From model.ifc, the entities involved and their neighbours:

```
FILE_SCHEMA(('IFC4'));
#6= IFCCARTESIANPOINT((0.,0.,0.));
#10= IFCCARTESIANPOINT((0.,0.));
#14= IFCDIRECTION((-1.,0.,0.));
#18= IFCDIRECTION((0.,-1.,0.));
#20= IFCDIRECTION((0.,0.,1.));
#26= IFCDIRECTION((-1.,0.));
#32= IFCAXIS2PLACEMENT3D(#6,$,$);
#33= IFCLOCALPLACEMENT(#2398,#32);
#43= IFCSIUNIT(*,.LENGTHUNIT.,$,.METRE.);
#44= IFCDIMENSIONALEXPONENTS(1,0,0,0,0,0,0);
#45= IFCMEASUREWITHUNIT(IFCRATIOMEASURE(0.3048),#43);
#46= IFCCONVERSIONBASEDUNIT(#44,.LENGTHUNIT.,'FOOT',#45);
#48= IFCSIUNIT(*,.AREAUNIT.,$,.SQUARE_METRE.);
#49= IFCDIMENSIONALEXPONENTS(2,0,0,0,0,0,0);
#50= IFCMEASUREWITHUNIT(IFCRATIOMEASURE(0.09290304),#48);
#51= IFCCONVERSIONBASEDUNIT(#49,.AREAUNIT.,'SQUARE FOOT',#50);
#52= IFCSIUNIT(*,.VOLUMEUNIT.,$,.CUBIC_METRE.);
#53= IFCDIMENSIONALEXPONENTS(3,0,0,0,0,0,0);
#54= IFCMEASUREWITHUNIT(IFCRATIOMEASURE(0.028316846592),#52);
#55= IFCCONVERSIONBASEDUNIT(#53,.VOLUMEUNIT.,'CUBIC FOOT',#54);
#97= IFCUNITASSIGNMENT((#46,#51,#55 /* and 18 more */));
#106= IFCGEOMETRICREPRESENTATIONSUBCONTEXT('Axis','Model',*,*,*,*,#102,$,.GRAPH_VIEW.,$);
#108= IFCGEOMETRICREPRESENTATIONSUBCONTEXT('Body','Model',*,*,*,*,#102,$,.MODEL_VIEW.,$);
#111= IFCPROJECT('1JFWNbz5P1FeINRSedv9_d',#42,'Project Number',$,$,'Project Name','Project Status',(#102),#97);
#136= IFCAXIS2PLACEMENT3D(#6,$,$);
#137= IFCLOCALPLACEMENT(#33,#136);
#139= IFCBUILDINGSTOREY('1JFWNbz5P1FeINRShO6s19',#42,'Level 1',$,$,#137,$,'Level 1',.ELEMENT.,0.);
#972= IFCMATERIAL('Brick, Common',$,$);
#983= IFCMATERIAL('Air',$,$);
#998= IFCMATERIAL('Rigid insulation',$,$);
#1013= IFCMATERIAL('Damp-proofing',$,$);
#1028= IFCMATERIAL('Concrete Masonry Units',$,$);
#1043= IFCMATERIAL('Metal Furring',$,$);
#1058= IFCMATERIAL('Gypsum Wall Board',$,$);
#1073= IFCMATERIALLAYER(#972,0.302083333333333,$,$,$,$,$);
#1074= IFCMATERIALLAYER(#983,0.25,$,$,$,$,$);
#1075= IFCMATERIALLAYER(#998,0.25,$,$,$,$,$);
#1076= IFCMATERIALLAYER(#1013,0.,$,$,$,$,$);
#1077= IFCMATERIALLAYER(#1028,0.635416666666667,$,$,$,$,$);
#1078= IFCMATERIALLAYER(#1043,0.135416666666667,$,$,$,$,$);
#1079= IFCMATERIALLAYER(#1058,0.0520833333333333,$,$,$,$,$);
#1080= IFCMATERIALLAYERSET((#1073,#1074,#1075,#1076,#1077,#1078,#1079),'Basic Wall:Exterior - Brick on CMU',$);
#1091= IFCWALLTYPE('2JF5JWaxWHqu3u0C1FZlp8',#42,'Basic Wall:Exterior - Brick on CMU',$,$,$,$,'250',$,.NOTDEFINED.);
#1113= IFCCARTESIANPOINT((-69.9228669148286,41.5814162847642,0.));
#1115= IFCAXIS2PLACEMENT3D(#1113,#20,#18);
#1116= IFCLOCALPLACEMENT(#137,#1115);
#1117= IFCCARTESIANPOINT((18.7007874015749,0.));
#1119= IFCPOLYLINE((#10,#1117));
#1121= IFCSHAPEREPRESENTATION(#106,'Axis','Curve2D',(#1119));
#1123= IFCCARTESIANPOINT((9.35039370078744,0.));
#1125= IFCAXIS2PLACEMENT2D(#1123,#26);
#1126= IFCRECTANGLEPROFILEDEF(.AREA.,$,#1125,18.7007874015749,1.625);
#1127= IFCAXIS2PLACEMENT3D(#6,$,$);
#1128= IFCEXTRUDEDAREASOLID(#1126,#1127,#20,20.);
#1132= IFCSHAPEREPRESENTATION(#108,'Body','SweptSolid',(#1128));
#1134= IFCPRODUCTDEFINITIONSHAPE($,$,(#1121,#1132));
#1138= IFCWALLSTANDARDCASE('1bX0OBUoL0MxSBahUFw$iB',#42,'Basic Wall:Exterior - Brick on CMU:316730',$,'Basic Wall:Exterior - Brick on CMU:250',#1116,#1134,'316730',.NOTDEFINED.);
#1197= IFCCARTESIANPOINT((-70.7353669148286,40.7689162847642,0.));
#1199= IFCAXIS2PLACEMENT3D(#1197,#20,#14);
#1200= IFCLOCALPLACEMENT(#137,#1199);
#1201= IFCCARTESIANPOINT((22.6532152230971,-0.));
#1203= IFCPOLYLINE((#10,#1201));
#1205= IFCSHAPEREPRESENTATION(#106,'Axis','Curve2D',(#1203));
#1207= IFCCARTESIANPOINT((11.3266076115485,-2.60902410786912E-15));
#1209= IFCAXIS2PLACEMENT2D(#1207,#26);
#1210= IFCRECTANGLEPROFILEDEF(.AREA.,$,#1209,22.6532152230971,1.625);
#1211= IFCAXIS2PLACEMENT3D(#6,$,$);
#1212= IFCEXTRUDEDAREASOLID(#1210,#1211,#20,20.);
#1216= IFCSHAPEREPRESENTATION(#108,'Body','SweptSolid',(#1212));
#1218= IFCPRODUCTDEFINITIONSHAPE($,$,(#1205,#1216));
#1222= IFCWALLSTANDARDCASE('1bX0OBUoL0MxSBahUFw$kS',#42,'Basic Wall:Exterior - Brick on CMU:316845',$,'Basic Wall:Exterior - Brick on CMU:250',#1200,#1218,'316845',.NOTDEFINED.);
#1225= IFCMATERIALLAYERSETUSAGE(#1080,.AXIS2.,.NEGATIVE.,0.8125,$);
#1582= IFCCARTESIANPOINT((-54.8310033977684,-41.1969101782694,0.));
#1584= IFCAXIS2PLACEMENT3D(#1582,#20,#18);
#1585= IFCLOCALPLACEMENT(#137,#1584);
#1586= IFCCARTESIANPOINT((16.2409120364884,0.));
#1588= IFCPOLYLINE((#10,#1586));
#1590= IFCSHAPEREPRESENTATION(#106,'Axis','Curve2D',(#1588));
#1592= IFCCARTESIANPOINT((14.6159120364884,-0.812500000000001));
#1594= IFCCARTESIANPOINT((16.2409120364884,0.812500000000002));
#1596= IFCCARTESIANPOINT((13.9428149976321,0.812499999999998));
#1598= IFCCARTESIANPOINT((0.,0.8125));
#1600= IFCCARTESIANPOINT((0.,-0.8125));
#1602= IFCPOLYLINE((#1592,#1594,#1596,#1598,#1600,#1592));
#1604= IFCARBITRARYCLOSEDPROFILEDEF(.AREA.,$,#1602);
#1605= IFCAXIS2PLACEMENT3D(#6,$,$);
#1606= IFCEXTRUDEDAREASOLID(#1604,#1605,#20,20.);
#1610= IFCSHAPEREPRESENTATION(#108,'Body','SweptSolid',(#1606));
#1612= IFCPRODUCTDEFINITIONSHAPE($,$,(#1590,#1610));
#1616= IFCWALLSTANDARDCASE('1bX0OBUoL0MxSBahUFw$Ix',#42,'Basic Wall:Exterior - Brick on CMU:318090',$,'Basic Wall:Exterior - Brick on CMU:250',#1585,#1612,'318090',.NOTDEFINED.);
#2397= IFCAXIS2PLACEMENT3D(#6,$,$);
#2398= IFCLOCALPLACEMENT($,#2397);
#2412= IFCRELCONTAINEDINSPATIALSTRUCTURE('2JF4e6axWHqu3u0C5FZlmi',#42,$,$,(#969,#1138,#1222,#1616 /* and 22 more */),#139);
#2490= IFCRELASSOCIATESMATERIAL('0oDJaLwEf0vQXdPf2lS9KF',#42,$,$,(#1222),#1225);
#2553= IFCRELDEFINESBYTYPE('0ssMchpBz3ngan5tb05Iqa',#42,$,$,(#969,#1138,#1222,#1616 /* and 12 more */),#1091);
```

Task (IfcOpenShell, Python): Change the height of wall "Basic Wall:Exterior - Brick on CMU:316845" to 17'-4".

```python
import ifcopenshell
import ifcopenshell.geom
import ifcopenshell.util.representation
import ifcopenshell.util.shape
import ifcopenshell.util.unit

model = ifcopenshell.open("model.ifc")
unit_scale = ifcopenshell.util.unit.calculate_unit_scale(model)
settings = ifcopenshell.geom.settings()


def volume(element):
    """Net volume in cubic metres, openings subtracted."""
    shape = ifcopenshell.geom.create_shape(settings, element)
    return ifcopenshell.util.shape.get_volume(shape.geometry)


wall = model.by_id(1222)
before = volume(wall)

body = ifcopenshell.util.representation.get_representation(wall, "Model", "Body")
solid = body.Items[0]
old_height = solid.Depth
solid.Depth = 208 * 0.0254 / unit_scale
after = volume(wall)

print(f"height {old_height:g} -> {solid.Depth:g}, volume {before:.3f} -> {after:.3f} m3")

model.write("model_rev.ifc")
```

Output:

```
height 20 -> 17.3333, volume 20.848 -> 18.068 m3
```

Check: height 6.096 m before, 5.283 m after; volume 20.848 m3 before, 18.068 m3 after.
